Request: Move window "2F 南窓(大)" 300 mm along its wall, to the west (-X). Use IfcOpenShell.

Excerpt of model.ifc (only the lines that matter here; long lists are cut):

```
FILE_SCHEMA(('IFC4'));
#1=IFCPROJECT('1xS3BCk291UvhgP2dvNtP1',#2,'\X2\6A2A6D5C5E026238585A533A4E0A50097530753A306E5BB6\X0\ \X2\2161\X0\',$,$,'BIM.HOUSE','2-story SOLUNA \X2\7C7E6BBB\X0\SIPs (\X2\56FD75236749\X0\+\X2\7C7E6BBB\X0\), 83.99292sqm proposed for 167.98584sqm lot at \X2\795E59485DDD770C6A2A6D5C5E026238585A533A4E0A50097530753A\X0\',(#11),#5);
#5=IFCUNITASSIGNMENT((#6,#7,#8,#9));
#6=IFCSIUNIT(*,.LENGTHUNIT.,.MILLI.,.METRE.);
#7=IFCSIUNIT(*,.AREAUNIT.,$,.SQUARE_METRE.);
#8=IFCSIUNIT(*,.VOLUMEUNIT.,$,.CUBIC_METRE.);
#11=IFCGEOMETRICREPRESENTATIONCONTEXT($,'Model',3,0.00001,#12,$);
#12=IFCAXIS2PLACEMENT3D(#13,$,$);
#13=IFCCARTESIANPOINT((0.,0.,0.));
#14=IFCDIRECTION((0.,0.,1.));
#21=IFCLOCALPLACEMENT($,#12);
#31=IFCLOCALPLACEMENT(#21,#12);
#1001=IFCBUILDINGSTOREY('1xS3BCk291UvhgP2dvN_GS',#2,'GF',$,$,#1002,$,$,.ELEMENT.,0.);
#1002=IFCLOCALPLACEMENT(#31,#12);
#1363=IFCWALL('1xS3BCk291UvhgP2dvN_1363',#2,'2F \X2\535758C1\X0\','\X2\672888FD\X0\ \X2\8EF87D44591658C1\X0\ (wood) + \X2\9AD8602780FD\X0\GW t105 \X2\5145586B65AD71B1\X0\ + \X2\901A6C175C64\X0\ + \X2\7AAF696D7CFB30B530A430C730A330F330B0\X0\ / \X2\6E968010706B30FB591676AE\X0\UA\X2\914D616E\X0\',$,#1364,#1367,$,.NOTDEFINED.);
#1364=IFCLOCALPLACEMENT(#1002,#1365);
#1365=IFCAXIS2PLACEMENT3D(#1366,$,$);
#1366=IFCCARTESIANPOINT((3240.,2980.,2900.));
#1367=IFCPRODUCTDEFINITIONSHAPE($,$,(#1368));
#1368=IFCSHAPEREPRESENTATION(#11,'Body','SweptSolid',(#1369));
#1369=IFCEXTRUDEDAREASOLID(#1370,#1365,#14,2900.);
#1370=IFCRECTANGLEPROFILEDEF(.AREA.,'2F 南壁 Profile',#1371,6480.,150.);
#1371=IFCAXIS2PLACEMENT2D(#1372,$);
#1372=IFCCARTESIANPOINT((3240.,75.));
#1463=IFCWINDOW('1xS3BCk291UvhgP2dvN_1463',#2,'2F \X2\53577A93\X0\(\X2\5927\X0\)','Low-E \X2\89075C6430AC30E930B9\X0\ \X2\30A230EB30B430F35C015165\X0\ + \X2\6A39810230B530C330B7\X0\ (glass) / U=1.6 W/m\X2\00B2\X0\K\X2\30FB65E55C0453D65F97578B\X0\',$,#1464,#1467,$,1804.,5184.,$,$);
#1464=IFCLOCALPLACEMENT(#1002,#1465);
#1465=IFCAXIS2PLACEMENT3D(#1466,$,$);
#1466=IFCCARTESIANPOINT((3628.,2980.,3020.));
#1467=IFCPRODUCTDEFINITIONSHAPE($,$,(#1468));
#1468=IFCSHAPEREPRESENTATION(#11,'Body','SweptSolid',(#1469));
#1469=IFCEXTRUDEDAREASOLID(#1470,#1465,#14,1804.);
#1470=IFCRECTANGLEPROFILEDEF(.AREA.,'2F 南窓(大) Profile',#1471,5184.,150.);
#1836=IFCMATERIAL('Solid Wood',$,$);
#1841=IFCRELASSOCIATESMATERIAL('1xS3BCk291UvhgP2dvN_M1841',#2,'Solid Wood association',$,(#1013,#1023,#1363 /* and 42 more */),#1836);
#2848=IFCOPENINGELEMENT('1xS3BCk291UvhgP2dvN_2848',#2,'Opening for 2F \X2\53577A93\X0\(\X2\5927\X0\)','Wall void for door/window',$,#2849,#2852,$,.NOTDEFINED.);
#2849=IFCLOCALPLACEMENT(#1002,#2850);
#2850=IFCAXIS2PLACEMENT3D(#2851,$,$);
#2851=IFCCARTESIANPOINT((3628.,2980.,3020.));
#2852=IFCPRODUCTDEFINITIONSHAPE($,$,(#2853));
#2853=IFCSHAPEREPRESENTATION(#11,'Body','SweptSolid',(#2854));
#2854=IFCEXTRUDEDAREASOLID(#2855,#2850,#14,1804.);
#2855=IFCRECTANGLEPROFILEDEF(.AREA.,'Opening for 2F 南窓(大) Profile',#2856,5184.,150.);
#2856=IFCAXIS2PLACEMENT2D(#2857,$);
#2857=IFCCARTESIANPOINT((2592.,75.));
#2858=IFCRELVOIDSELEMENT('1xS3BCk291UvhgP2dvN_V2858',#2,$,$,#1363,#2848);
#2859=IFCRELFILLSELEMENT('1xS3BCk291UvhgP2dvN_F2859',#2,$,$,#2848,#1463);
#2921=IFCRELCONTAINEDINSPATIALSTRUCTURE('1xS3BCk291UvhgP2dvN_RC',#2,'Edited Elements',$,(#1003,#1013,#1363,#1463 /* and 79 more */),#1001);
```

```python
import ifcopenshell
import ifcopenshell.api.geometry
import ifcopenshell.util.placement

model = ifcopenshell.open("model.ifc")

window = model.by_guid("1xS3BCk291UvhgP2dvN_1463")
opening = window.FillsVoids[0].RelatingOpeningElement
wall = opening.VoidsElements[0].RelatingBuildingElement

wall_matrix = ifcopenshell.util.placement.get_local_placement(wall.ObjectPlacement)
shift = wall_matrix[:3, 0] * -300.0
before = ifcopenshell.util.placement.get_local_placement(window.ObjectPlacement)[:3, 3].copy()

# The window is not placed relative to its opening, so move both.
for product in (opening, window):
    matrix = ifcopenshell.util.placement.get_local_placement(product.ObjectPlacement)
    matrix[:3, 3] += shift
    ifcopenshell.api.geometry.edit_object_placement(model, product=product, matrix=matrix, is_si=False)

after = ifcopenshell.util.placement.get_local_placement(window.ObjectPlacement)[:3, 3]
print("window moved by", (after - before).round(3) + 0.0)

model.write("model-out.ifc")
```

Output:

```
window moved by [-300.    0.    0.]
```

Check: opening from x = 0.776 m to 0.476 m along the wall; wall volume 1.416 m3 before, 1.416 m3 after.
